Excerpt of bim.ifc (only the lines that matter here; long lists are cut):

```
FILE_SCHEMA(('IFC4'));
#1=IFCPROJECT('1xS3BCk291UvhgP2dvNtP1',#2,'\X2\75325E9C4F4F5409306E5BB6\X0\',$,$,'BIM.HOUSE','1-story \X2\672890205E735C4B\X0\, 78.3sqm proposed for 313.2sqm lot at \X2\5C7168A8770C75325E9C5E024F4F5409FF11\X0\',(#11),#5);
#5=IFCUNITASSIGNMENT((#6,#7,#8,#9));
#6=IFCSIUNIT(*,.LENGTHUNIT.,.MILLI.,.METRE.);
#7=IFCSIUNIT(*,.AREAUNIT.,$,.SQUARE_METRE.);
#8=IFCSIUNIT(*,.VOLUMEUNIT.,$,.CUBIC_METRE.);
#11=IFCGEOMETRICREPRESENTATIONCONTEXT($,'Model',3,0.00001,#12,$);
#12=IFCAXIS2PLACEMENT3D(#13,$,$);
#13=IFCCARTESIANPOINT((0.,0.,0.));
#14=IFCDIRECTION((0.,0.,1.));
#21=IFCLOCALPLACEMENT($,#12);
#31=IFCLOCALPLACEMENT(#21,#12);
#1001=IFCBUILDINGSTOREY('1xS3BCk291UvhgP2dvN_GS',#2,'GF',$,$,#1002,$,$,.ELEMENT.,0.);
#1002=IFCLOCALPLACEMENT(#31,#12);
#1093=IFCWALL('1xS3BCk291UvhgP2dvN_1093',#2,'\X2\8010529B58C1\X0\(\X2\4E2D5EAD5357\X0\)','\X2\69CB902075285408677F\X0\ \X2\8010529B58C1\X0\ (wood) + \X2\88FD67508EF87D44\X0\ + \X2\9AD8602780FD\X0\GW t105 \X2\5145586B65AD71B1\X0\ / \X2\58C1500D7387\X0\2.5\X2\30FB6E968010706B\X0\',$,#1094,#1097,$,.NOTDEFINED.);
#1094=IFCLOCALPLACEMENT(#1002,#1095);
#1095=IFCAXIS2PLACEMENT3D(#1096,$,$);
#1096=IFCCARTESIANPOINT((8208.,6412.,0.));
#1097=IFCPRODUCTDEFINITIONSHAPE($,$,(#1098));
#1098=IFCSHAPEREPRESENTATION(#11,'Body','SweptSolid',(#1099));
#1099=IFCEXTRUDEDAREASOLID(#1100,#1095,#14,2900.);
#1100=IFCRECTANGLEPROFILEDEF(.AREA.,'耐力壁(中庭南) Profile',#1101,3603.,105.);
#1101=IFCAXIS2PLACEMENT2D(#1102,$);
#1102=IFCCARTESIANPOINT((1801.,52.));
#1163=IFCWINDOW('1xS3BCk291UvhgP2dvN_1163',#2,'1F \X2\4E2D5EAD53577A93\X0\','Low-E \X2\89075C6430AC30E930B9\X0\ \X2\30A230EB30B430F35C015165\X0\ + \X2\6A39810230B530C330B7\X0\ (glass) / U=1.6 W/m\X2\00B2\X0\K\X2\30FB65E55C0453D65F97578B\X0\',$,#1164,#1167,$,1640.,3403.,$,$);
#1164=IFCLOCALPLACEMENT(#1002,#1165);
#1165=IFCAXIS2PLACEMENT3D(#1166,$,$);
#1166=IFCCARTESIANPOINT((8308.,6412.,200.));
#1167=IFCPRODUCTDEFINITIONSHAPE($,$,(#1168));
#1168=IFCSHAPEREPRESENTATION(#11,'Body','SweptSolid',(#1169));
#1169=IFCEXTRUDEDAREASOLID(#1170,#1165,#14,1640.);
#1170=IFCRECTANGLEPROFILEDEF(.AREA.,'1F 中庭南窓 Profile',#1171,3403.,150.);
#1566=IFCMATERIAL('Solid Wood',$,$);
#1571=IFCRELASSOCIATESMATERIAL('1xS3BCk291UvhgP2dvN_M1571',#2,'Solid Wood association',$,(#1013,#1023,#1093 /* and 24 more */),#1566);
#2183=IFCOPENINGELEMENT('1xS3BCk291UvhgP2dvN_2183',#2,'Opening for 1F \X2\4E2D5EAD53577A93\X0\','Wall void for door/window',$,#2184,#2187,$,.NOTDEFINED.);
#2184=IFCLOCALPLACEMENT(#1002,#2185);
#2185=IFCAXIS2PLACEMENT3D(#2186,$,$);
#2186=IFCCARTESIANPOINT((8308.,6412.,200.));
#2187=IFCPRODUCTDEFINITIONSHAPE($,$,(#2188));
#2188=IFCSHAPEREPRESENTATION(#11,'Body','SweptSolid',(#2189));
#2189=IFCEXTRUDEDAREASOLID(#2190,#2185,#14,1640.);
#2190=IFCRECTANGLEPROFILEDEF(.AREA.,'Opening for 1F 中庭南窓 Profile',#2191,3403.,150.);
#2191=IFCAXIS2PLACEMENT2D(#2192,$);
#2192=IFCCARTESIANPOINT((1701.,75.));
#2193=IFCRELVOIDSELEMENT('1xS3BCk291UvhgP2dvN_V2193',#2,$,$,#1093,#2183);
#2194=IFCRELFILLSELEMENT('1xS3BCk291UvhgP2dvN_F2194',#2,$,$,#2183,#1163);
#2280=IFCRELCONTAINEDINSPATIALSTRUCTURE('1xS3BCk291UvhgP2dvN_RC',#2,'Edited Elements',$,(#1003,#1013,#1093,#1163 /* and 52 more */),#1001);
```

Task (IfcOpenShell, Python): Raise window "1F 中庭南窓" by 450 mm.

```python
import numpy as np
import ifcopenshell
import ifcopenshell.api.geometry
import ifcopenshell.util.placement
import ifcopenshell.util.unit

model = ifcopenshell.open("bim.ifc")
unit_scale = ifcopenshell.util.unit.calculate_unit_scale(model)

window = model.by_id(1163)
opening = window.FillsVoids[0].RelatingOpeningElement
dz = 0.45 / unit_scale

shift = np.array([0.0, 0.0, dz])
# The window is not placed relative to its opening, so move both.
for product in (opening, window):
    matrix = ifcopenshell.util.placement.get_local_placement(product.ObjectPlacement)
    matrix[:3, 3] += shift
    ifcopenshell.api.geometry.edit_object_placement(model, product=product, matrix=matrix, is_si=False)

print(f"moved by {dz * unit_scale:+.3f} m")

model.write("bim_updated.ifc")
```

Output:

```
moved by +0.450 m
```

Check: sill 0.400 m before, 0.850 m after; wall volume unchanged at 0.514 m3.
